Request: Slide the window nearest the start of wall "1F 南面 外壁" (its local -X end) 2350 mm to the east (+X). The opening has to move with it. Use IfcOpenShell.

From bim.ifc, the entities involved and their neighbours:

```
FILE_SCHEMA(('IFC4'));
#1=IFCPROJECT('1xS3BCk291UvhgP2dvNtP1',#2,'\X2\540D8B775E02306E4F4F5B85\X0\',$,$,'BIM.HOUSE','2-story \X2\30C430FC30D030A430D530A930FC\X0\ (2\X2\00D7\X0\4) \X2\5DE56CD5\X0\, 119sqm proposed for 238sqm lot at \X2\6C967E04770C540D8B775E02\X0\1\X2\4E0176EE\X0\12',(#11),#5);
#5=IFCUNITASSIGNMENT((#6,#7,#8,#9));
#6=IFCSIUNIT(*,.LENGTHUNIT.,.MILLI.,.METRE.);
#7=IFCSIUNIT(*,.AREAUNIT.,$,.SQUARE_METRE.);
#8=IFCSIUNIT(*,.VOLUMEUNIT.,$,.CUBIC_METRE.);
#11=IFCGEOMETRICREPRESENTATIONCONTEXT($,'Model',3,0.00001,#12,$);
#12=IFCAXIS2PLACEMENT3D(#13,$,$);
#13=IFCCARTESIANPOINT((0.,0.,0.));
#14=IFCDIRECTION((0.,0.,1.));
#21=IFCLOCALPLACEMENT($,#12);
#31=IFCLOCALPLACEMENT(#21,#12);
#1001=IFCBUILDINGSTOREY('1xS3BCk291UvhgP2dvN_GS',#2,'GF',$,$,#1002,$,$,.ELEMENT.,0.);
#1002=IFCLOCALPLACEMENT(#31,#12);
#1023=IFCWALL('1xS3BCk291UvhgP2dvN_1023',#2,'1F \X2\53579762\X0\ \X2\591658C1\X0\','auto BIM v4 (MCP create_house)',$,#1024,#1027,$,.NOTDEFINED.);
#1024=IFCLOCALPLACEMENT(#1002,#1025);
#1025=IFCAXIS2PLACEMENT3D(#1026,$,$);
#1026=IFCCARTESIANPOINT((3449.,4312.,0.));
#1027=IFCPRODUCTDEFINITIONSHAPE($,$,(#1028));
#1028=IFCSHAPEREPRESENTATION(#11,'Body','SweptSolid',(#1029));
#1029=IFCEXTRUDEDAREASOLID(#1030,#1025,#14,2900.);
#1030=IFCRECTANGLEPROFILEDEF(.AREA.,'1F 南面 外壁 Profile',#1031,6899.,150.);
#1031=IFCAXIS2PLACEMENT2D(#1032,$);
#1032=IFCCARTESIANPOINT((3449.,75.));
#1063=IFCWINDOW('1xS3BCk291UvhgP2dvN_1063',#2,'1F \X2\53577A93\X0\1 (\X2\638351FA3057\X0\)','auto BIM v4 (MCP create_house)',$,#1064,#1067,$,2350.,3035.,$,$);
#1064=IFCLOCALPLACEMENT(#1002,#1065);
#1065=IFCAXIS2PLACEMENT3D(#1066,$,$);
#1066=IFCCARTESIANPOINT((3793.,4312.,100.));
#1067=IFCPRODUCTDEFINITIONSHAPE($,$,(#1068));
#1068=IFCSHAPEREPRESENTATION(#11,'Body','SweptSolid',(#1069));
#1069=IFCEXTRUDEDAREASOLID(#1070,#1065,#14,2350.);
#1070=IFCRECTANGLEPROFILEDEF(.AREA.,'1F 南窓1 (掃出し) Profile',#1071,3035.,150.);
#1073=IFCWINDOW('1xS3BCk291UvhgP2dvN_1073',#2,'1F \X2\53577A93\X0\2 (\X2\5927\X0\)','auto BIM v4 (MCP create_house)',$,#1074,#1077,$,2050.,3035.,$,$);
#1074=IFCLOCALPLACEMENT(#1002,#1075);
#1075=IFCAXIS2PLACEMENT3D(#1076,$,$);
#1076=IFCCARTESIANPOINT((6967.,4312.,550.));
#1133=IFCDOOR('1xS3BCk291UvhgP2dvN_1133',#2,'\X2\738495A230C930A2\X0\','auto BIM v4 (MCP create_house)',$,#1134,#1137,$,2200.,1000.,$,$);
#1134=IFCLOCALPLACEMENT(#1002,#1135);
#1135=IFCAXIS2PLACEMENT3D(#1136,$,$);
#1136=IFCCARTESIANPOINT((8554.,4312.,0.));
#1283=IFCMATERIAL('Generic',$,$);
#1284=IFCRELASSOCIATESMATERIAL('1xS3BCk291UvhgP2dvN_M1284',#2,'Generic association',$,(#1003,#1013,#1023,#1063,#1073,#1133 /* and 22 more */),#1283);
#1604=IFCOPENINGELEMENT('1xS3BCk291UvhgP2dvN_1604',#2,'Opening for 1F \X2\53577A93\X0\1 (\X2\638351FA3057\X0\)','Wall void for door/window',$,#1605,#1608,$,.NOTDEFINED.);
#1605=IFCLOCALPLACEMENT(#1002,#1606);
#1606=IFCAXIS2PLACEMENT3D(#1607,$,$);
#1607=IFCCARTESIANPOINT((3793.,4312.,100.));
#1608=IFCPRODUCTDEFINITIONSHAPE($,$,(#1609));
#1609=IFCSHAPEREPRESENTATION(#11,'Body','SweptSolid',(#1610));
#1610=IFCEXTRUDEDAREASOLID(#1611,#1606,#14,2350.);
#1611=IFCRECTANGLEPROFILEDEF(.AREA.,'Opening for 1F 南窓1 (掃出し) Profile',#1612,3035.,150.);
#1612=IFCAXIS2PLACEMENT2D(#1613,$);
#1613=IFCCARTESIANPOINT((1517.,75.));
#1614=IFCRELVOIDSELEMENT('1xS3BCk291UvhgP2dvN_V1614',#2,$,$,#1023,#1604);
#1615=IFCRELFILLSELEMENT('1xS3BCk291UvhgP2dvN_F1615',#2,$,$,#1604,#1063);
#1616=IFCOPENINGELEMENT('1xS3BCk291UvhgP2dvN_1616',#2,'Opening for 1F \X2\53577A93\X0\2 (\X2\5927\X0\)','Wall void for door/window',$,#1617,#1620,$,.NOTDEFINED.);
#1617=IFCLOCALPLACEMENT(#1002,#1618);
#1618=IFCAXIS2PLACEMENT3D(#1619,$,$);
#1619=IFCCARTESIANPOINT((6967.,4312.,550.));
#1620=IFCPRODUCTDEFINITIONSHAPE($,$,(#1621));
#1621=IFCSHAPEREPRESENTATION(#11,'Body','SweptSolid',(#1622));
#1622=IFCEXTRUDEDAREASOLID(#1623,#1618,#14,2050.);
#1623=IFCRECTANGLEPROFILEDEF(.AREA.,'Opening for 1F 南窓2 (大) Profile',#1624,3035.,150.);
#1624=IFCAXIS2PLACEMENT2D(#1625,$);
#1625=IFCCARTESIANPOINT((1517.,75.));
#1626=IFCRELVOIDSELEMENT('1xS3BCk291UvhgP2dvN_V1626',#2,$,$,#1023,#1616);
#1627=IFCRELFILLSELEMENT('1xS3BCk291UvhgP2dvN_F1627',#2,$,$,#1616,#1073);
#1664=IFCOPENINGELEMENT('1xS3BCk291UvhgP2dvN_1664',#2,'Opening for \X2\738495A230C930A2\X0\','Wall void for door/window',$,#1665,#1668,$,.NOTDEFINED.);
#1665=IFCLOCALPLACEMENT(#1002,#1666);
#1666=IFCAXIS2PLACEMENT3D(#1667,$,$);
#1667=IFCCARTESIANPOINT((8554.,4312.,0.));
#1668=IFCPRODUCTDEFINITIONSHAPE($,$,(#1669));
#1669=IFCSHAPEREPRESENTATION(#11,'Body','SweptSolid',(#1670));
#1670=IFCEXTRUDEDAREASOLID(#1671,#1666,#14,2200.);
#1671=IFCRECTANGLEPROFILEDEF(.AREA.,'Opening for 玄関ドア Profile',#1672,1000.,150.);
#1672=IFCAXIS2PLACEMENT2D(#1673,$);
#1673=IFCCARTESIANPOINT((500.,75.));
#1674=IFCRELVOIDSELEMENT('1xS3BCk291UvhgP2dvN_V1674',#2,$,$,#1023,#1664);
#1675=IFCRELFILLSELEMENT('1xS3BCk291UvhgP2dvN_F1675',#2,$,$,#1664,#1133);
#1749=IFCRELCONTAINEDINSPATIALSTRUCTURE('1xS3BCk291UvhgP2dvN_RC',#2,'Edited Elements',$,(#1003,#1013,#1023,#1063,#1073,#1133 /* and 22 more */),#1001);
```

```python
import ifcopenshell
import ifcopenshell.api.geometry
import ifcopenshell.util.placement
import ifcopenshell.util.unit

model = ifcopenshell.open("bim.ifc")
unit_scale = ifcopenshell.util.unit.calculate_unit_scale(model)

window = model.by_guid("1xS3BCk291UvhgP2dvN_1063")
opening = window.FillsVoids[0].RelatingOpeningElement
wall = opening.VoidsElements[0].RelatingBuildingElement

wall_matrix = ifcopenshell.util.placement.get_local_placement(wall.ObjectPlacement)
shift = wall_matrix[:3, 0] * 2.35 / unit_scale
before = ifcopenshell.util.placement.get_local_placement(window.ObjectPlacement)[:3, 3].copy()

# The window is not placed relative to its opening, so move both.
for product in (opening, window):
    matrix = ifcopenshell.util.placement.get_local_placement(product.ObjectPlacement)
    matrix[:3, 3] += shift
    ifcopenshell.api.geometry.edit_object_placement(model, product=product, matrix=matrix, is_si=False)

after = ifcopenshell.util.placement.get_local_placement(window.ObjectPlacement)[:3, 3]
print("window moved by", (after - before).round(3) + 0.0)

model.write("bim_edited.ifc")
```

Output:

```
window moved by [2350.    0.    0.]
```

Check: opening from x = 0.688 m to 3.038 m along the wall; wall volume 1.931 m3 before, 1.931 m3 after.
